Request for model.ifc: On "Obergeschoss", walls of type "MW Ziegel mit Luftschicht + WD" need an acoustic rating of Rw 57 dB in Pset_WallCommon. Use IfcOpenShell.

First a look at what the model holds.

```python
import ifcopenshell
import ifcopenshell.util.element

model = ifcopenshell.open("model.ifc")
print(model.schema)
storey = next(s for s in model.by_type("IfcBuildingStorey") if s.Name == "Obergeschoss")
walls = [e for e in ifcopenshell.util.element.get_decomposition(storey) if e.is_a("IfcWall")]
seen = {}
for e in walls:
    element_type = ifcopenshell.util.element.get_type(e)
    key = (element_type.Name if element_type != e and element_type else None, ifcopenshell.util.element.get_pset(e, "Pset_WallCommon", "AcousticRating"))
    seen[key] = seen.get(key, 0) + 1
for (name, value), count in sorted(seen.items(), key=str):
    print(count, "x", name, "|", value)
```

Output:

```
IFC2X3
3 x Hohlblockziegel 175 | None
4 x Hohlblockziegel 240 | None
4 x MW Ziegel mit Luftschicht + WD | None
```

```python
import ifcopenshell
import ifcopenshell.api.pset
import ifcopenshell.util.element

model = ifcopenshell.open("model.ifc")

storey = next(s for s in model.by_type("IfcBuildingStorey") if s.Name == "Obergeschoss")
walls = [e for e in ifcopenshell.util.element.get_decomposition(storey) if e.is_a("IfcWall")]

count = 0
for e in walls:
    element_type = ifcopenshell.util.element.get_type(e)
    if element_type in (None, e) or element_type.Name != "MW Ziegel mit Luftschicht + WD":
        continue
    # add_pset returns the element's existing set when there is one.
    pset = ifcopenshell.api.pset.add_pset(model, product=e, name="Pset_WallCommon")
    ifcopenshell.api.pset.edit_pset(model, pset=pset, properties={"AcousticRating": "Rw 57 dB"})
    count += 1

print(count, "walls updated")

model.write("model_edited.ifc")
```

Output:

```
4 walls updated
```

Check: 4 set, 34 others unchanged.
